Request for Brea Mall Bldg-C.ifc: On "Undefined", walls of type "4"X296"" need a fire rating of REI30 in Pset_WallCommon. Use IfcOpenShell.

First a look at what the model holds.

```python
import ifcopenshell
import ifcopenshell.util.element

model = ifcopenshell.open("Brea Mall Bldg-C.ifc")
print(model.schema)
storey = next(s for s in model.by_type("IfcBuildingStorey") if s.Name == "Undefined")
walls = [e for e in ifcopenshell.util.element.get_decomposition(storey) if e.is_a("IfcWall")]
seen = {}
for e in walls:
    element_type = ifcopenshell.util.element.get_type(e)
    key = (element_type.Name if element_type != e and element_type else None, ifcopenshell.util.element.get_pset(e, "Pset_WallCommon", "FireRating"))
    seen[key] = seen.get(key, 0) + 1
for (name, value), count in sorted(seen.items(), key=str):
    print(count, "x", name, "|", value)
```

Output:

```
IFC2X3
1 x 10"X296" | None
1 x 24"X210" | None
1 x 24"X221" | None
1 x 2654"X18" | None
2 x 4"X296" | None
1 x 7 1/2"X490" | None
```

```python
import ifcopenshell
import ifcopenshell.api.pset
import ifcopenshell.util.element

model = ifcopenshell.open("Brea Mall Bldg-C.ifc")

storey = next(s for s in model.by_type("IfcBuildingStorey") if s.Name == "Undefined")
walls = [e for e in ifcopenshell.util.element.get_decomposition(storey) if e.is_a("IfcWall")]

count = 0
for e in walls:
    element_type = ifcopenshell.util.element.get_type(e)
    if element_type in (None, e) or element_type.Name != '4"X296"':
        continue
    # add_pset returns the element's existing set when there is one.
    pset = ifcopenshell.api.pset.add_pset(model, product=e, name="Pset_WallCommon")
    ifcopenshell.api.pset.edit_pset(model, pset=pset, properties={"FireRating": "REI30"})
    count += 1

print(count, "walls updated")

model.write("Brea Mall Bldg-C_v2.ifc")
```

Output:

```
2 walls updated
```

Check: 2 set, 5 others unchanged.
